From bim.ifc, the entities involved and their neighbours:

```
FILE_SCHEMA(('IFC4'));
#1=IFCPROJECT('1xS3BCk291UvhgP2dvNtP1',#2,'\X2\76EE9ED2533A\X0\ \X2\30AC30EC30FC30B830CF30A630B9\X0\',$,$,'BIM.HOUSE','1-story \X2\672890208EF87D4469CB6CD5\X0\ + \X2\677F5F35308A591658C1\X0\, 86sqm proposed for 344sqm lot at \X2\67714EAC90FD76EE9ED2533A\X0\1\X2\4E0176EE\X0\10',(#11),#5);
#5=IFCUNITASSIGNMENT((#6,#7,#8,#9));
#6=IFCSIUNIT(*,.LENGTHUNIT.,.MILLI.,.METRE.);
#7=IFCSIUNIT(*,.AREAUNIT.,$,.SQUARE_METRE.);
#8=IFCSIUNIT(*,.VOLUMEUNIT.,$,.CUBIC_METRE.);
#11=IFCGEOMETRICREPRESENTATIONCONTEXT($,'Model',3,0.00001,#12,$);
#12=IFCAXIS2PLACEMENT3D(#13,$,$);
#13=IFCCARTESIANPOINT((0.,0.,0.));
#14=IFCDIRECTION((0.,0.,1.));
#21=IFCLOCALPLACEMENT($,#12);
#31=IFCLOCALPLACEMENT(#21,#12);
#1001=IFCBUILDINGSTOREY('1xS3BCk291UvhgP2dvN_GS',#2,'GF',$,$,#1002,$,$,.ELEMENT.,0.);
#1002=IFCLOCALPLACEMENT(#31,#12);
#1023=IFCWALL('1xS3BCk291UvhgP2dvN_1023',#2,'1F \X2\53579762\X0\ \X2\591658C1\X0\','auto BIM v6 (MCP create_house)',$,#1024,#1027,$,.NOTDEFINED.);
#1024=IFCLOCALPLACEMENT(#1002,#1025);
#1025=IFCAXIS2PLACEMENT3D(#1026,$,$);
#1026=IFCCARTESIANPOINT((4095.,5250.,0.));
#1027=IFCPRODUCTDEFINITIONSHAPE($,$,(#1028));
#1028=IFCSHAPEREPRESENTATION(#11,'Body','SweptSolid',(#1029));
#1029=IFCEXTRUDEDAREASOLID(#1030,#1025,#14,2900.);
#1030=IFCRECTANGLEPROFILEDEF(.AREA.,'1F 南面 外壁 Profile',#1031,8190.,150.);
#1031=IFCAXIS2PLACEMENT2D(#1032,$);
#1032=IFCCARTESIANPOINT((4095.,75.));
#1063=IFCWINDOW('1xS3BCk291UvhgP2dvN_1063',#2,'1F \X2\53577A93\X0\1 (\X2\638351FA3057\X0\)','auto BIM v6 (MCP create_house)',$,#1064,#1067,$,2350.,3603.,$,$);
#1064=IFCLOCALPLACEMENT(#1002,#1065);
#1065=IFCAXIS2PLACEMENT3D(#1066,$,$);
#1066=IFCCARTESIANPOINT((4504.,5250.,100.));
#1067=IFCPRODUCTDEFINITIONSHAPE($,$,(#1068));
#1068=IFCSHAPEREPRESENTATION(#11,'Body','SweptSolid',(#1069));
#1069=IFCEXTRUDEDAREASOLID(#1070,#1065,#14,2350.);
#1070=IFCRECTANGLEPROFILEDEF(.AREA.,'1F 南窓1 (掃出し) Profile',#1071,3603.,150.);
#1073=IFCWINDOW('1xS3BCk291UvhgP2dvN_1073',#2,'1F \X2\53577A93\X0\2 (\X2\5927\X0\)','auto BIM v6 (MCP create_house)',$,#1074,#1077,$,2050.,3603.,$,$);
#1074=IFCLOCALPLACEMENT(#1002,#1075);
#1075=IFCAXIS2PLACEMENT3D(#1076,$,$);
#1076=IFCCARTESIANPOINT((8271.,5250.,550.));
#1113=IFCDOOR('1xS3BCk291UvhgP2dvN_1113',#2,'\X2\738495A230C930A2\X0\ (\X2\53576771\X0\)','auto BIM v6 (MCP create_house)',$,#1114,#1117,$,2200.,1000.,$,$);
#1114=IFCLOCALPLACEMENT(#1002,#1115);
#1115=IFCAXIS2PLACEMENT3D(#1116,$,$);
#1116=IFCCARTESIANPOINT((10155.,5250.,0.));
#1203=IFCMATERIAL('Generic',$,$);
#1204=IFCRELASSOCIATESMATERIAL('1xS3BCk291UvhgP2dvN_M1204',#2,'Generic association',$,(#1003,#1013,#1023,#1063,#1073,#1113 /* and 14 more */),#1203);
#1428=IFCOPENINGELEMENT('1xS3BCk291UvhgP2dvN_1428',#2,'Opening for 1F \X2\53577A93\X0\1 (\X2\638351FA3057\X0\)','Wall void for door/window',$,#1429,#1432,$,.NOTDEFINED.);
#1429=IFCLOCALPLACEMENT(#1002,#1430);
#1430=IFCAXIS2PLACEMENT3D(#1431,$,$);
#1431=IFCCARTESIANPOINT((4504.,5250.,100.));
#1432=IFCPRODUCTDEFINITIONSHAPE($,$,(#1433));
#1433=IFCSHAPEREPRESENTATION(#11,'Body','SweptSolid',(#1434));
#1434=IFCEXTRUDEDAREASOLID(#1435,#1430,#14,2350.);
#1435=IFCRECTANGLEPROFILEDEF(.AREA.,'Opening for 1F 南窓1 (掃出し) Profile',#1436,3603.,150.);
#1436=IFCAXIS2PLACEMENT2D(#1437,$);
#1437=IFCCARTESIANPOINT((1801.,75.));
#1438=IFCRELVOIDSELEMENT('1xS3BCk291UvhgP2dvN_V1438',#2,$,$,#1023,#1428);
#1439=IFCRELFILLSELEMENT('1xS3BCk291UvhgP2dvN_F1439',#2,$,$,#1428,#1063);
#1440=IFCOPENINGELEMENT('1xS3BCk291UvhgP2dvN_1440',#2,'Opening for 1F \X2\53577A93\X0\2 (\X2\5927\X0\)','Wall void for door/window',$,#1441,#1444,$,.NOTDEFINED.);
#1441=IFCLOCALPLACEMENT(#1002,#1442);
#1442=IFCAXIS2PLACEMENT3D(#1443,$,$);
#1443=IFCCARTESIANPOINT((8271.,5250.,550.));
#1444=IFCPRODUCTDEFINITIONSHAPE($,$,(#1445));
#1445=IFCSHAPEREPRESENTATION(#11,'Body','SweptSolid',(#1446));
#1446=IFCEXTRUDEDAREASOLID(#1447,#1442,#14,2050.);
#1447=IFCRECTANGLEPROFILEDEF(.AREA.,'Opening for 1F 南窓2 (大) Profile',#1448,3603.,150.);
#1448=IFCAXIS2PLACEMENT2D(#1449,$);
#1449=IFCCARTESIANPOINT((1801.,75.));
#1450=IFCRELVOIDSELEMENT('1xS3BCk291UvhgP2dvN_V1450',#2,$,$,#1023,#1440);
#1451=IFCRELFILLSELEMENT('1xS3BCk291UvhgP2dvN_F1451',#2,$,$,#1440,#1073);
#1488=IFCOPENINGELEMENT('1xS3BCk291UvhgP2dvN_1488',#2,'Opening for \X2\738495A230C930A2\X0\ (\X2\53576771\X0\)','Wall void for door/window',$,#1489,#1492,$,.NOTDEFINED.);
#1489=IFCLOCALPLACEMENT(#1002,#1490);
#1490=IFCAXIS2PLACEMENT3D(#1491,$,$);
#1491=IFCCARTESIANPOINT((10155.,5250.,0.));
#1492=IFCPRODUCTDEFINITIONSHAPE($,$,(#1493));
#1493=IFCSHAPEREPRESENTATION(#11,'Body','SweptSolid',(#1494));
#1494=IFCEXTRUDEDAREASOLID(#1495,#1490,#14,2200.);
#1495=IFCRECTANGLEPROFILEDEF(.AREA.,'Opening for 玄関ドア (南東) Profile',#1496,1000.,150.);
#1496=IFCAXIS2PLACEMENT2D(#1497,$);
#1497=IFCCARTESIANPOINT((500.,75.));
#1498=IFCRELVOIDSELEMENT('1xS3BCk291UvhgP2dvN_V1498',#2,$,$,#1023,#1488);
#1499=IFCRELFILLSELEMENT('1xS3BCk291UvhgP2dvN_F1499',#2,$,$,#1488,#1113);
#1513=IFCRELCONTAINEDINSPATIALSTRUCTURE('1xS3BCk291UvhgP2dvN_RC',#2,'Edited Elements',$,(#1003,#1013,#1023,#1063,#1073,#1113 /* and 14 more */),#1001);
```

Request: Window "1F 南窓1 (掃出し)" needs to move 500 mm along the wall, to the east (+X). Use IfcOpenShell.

```python
import ifcopenshell
import ifcopenshell.api.geometry
import ifcopenshell.util.placement

model = ifcopenshell.open("bim.ifc")

window = model.by_id(1063)
opening = window.FillsVoids[0].RelatingOpeningElement
wall = opening.VoidsElements[0].RelatingBuildingElement

wall_matrix = ifcopenshell.util.placement.get_local_placement(wall.ObjectPlacement)
shift = wall_matrix[:3, 0] * 500.0
before = ifcopenshell.util.placement.get_local_placement(window.ObjectPlacement)[:3, 3].copy()

# The window is not placed relative to its opening, so move both.
for product in (opening, window):
    matrix = ifcopenshell.util.placement.get_local_placement(product.ObjectPlacement)
    matrix[:3, 3] += shift
    ifcopenshell.api.geometry.edit_object_placement(model, product=product, matrix=matrix, is_si=False)

after = ifcopenshell.util.placement.get_local_placement(window.ObjectPlacement)[:3, 3]
print("window moved by", (after - before).round(3) + 0.0)

model.write("bim_edited.ifc")
```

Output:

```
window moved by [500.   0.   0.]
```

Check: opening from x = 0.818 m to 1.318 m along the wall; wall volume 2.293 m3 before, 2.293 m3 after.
